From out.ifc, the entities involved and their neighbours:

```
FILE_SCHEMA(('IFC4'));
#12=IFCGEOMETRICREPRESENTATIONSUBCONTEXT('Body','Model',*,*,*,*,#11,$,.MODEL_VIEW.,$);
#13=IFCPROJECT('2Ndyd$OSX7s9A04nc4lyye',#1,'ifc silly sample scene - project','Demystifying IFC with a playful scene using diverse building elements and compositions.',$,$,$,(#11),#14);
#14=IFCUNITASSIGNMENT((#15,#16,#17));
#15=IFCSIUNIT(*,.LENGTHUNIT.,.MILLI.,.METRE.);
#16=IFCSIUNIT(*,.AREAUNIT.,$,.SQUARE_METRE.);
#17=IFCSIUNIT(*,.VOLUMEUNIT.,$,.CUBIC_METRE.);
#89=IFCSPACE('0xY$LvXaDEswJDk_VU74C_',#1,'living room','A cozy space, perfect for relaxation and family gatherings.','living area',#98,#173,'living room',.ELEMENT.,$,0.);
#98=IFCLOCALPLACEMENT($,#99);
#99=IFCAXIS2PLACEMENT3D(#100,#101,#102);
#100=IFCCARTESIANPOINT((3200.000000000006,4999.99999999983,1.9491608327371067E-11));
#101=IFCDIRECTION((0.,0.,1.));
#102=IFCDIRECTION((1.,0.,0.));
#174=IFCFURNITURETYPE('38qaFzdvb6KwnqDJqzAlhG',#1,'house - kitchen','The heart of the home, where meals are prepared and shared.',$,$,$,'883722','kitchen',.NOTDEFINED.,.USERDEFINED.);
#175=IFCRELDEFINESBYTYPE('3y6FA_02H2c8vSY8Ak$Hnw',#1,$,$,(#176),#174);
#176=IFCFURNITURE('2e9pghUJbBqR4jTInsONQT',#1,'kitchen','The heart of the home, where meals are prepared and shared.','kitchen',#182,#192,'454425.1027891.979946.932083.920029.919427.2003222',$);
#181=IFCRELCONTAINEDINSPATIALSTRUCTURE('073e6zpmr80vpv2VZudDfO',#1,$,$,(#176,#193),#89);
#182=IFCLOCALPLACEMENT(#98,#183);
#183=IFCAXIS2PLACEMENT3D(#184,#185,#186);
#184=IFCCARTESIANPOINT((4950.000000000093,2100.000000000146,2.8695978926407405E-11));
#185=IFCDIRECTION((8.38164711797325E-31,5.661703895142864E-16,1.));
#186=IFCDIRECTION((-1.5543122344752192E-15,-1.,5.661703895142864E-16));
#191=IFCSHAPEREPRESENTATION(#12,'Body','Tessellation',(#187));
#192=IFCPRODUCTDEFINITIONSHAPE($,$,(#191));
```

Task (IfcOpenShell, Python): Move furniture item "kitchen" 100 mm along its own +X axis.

```python
import ifcopenshell
import ifcopenshell.api.geometry
import ifcopenshell.util.placement
import ifcopenshell.util.unit

model = ifcopenshell.open("out.ifc")
unit_scale = ifcopenshell.util.unit.calculate_unit_scale(model)

item = model.by_guid("2e9pghUJbBqR4jTInsONQT")
matrix = ifcopenshell.util.placement.get_local_placement(item.ObjectPlacement)
matrix[:3, 3] += matrix[:3, 0] * 0.1 / unit_scale
ifcopenshell.api.geometry.edit_object_placement(model, product=item, matrix=matrix, is_si=False)

print(ifcopenshell.util.placement.get_local_placement(item.ObjectPlacement).round(3) + 0.0)

model.write("out_edited.ifc")
```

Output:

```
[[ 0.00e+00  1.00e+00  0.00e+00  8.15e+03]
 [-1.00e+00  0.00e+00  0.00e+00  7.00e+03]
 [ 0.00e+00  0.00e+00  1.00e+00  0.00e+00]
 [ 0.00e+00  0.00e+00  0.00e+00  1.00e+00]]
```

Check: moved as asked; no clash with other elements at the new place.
